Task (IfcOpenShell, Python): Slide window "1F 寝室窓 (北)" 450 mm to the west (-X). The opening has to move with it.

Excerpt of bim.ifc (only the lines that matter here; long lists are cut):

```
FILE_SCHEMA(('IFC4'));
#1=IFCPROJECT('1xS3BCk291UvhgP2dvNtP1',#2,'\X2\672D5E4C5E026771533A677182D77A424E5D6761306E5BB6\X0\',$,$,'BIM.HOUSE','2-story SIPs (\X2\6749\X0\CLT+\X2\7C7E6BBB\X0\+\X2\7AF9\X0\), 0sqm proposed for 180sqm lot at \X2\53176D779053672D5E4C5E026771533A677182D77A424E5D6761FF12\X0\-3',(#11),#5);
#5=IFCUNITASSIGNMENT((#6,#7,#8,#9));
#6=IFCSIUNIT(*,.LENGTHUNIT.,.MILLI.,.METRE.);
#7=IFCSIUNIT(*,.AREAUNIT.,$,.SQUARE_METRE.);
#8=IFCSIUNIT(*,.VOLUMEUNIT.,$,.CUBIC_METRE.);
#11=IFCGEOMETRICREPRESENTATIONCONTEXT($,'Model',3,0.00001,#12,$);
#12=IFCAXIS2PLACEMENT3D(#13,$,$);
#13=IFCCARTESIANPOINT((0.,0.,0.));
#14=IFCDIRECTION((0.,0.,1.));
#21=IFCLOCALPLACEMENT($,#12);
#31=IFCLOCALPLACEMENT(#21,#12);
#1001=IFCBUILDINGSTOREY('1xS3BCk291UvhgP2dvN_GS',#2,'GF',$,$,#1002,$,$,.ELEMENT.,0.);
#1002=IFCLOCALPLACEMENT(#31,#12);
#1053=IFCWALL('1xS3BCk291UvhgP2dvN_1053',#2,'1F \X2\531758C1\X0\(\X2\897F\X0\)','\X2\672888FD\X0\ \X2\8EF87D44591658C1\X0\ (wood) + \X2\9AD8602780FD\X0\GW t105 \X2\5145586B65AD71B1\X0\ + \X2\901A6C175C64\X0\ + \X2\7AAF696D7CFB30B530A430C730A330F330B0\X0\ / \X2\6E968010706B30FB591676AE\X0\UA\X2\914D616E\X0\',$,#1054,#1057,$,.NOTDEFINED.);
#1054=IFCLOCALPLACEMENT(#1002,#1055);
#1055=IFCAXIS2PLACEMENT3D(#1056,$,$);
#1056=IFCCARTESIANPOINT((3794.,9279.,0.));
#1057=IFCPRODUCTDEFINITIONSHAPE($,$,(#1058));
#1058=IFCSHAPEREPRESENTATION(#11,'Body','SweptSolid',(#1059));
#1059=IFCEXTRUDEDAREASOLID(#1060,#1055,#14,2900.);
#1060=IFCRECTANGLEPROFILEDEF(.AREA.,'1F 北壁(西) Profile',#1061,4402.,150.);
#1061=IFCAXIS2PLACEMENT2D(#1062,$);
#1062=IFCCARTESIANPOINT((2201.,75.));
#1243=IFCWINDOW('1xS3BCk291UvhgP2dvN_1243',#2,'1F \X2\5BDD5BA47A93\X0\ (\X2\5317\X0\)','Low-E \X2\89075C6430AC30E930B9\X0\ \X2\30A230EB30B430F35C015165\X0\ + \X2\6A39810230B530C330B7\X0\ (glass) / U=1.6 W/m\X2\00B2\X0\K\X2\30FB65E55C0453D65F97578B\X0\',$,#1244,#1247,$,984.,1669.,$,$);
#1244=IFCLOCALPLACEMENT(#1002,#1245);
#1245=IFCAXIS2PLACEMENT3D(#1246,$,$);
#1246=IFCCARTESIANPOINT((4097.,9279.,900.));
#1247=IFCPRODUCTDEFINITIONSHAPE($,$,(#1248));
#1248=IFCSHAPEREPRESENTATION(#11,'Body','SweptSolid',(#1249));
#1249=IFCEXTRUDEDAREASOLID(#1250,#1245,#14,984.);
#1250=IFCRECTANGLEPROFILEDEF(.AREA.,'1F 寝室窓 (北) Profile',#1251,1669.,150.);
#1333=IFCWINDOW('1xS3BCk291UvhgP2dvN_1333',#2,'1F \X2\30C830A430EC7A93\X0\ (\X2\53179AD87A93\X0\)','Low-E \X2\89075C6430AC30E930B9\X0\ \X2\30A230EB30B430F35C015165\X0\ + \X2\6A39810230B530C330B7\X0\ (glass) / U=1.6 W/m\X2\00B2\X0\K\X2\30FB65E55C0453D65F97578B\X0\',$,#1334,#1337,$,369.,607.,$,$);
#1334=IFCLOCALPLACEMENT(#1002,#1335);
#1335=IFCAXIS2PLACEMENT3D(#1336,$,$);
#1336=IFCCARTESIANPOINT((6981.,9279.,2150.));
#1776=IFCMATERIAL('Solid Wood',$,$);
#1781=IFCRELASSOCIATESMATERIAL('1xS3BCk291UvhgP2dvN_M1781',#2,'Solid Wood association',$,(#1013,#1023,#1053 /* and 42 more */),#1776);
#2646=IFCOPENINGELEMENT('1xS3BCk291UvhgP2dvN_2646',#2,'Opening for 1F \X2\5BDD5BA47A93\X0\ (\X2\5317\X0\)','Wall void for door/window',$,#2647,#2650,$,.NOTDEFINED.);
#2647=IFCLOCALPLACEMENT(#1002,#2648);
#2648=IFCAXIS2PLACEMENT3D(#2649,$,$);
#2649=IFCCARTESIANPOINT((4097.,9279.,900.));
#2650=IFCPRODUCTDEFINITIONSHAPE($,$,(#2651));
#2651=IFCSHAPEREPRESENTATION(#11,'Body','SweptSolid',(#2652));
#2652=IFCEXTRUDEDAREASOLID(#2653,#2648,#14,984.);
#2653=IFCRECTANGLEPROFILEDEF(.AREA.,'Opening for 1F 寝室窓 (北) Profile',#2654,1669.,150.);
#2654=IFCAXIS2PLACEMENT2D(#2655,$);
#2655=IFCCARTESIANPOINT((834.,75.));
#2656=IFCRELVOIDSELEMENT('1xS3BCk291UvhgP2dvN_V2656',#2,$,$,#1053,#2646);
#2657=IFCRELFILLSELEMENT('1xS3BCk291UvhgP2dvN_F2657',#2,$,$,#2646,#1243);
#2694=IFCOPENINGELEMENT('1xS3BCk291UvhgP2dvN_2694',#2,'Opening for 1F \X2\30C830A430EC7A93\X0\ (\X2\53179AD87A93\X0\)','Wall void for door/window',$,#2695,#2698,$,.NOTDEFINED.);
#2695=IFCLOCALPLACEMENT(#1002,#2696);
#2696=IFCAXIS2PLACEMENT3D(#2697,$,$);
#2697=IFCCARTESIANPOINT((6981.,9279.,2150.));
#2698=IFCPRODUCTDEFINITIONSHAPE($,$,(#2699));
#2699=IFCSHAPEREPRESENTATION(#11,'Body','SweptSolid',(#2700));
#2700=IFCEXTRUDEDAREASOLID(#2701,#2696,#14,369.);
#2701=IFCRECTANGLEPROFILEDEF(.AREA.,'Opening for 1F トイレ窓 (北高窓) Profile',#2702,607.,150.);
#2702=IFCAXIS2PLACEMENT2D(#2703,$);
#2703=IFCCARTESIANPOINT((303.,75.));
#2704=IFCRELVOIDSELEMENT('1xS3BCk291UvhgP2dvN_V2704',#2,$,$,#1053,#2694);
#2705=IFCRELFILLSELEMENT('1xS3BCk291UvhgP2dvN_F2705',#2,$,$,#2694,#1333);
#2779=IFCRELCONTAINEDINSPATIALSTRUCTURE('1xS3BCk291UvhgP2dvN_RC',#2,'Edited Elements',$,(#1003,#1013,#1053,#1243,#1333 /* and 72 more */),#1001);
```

```python
import ifcopenshell
import ifcopenshell.api.geometry
import ifcopenshell.util.placement
import ifcopenshell.util.unit

model = ifcopenshell.open("bim.ifc")
unit_scale = ifcopenshell.util.unit.calculate_unit_scale(model)

window = model.by_guid("1xS3BCk291UvhgP2dvN_1243")
opening = window.FillsVoids[0].RelatingOpeningElement
wall = opening.VoidsElements[0].RelatingBuildingElement

wall_matrix = ifcopenshell.util.placement.get_local_placement(wall.ObjectPlacement)
shift = wall_matrix[:3, 0] * -0.45 / unit_scale
before = ifcopenshell.util.placement.get_local_placement(window.ObjectPlacement)[:3, 3].copy()

# The window is not placed relative to its opening, so move both.
for product in (opening, window):
    matrix = ifcopenshell.util.placement.get_local_placement(product.ObjectPlacement)
    matrix[:3, 3] += shift
    ifcopenshell.api.geometry.edit_object_placement(model, product=product, matrix=matrix, is_si=False)

after = ifcopenshell.util.placement.get_local_placement(window.ObjectPlacement)[:3, 3]
print("window moved by", (after - before).round(3) + 0.0)

model.write("bim_v2.ifc")
```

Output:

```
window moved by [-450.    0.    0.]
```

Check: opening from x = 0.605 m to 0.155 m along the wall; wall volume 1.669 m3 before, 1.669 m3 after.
